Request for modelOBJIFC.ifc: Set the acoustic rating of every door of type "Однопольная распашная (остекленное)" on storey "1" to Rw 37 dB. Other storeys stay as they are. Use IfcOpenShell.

First a look at what the model holds.

```python
import ifcopenshell
import ifcopenshell.util.element

model = ifcopenshell.open("modelOBJIFC.ifc")
print(model.schema)
storey = next(s for s in model.by_type("IfcBuildingStorey") if s.Name == "1")
doors = [e for e in ifcopenshell.util.element.get_decomposition(storey) if e.is_a("IfcDoor")]
seen = {}
for e in doors:
    element_type = ifcopenshell.util.element.get_type(e)
    key = (element_type.Name if element_type != e and element_type else None, ifcopenshell.util.element.get_pset(e, "Pset_DoorCommon", "AcousticRating"))
    seen[key] = seen.get(key, 0) + 1
for (name, value), count in sorted(seen.items(), key=str):
    print(count, "x", name, "|", value)
```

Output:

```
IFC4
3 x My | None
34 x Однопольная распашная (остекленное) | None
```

```python
import ifcopenshell
import ifcopenshell.api.pset
import ifcopenshell.util.element

model = ifcopenshell.open("modelOBJIFC.ifc")

storey = next(s for s in model.by_type("IfcBuildingStorey") if s.Name == "1")
doors = [e for e in ifcopenshell.util.element.get_decomposition(storey) if e.is_a("IfcDoor")]

count = 0
for e in doors:
    element_type = ifcopenshell.util.element.get_type(e)
    if element_type in (None, e) or element_type.Name != "Однопольная распашная (остекленное)":
        continue
    # add_pset returns the element's existing set when there is one.
    pset = ifcopenshell.api.pset.add_pset(model, product=e, name="Pset_DoorCommon")
    ifcopenshell.api.pset.edit_pset(model, pset=pset, properties={"AcousticRating": "Rw 37 dB"})
    count += 1

print(count, "doors updated")

model.write("modelOBJIFC_updated.ifc")
```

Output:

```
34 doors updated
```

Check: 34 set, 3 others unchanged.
